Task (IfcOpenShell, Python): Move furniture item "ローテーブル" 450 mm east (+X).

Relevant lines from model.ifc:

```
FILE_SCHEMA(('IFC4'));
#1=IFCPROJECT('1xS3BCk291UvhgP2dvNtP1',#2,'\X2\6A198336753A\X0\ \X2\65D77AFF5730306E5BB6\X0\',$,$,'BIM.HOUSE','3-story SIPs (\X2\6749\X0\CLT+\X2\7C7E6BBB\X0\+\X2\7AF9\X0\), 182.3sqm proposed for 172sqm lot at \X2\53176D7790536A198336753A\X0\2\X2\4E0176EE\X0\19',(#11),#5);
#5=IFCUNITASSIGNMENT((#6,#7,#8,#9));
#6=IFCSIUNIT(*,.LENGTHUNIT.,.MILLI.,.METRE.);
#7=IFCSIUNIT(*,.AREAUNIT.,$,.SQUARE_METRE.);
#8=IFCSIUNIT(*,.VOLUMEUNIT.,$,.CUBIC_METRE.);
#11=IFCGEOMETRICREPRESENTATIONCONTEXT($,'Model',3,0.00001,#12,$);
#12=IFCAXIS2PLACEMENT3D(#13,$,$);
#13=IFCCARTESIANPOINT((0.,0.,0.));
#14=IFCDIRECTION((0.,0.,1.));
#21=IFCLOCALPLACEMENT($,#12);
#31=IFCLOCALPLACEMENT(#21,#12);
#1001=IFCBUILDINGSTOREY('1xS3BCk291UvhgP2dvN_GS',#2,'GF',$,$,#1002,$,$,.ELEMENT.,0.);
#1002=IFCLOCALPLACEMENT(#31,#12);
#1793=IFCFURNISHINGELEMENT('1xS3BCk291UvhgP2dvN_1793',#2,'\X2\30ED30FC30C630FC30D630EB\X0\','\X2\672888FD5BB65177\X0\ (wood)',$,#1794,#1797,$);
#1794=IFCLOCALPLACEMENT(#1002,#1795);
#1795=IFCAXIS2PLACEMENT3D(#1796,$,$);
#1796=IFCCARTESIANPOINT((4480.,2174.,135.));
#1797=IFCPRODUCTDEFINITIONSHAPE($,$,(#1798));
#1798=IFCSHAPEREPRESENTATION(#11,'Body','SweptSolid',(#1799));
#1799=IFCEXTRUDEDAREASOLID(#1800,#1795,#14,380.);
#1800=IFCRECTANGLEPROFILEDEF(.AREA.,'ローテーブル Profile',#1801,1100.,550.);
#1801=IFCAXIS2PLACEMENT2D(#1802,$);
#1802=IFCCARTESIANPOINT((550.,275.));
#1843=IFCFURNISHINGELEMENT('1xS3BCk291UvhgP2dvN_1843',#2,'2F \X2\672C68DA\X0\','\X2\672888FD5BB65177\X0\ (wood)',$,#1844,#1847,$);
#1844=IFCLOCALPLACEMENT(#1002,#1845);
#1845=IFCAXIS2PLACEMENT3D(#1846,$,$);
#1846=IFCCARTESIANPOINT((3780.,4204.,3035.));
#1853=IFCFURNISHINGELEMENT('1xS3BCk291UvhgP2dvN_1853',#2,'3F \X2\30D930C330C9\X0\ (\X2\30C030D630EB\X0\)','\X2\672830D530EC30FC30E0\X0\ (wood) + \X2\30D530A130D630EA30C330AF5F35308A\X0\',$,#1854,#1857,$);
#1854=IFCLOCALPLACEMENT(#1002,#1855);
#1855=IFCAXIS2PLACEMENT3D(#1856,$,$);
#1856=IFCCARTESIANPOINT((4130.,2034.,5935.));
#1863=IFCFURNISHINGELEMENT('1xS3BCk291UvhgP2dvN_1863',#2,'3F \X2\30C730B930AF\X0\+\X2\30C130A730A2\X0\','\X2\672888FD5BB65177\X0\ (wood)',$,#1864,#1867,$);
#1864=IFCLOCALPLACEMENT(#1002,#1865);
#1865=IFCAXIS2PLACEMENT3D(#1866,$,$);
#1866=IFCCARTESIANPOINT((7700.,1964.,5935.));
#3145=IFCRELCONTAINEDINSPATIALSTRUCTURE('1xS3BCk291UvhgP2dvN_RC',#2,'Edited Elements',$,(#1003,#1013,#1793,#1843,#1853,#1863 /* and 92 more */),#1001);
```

```python
import ifcopenshell
import ifcopenshell.api.geometry
import ifcopenshell.util.placement
import ifcopenshell.util.unit

model = ifcopenshell.open("model.ifc")
unit_scale = ifcopenshell.util.unit.calculate_unit_scale(model)

item = model.by_guid("1xS3BCk291UvhgP2dvN_1793")
matrix = ifcopenshell.util.placement.get_local_placement(item.ObjectPlacement)
matrix[0, 3] += 0.45 / unit_scale
ifcopenshell.api.geometry.edit_object_placement(model, product=item, matrix=matrix, is_si=False)

print(ifcopenshell.util.placement.get_local_placement(item.ObjectPlacement).round(3) + 0.0)

model.write("model_rev.ifc")
```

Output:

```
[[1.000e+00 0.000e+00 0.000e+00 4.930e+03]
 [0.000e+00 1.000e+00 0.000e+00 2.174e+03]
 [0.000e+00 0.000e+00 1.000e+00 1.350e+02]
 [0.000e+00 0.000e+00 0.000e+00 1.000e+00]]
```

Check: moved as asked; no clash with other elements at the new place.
